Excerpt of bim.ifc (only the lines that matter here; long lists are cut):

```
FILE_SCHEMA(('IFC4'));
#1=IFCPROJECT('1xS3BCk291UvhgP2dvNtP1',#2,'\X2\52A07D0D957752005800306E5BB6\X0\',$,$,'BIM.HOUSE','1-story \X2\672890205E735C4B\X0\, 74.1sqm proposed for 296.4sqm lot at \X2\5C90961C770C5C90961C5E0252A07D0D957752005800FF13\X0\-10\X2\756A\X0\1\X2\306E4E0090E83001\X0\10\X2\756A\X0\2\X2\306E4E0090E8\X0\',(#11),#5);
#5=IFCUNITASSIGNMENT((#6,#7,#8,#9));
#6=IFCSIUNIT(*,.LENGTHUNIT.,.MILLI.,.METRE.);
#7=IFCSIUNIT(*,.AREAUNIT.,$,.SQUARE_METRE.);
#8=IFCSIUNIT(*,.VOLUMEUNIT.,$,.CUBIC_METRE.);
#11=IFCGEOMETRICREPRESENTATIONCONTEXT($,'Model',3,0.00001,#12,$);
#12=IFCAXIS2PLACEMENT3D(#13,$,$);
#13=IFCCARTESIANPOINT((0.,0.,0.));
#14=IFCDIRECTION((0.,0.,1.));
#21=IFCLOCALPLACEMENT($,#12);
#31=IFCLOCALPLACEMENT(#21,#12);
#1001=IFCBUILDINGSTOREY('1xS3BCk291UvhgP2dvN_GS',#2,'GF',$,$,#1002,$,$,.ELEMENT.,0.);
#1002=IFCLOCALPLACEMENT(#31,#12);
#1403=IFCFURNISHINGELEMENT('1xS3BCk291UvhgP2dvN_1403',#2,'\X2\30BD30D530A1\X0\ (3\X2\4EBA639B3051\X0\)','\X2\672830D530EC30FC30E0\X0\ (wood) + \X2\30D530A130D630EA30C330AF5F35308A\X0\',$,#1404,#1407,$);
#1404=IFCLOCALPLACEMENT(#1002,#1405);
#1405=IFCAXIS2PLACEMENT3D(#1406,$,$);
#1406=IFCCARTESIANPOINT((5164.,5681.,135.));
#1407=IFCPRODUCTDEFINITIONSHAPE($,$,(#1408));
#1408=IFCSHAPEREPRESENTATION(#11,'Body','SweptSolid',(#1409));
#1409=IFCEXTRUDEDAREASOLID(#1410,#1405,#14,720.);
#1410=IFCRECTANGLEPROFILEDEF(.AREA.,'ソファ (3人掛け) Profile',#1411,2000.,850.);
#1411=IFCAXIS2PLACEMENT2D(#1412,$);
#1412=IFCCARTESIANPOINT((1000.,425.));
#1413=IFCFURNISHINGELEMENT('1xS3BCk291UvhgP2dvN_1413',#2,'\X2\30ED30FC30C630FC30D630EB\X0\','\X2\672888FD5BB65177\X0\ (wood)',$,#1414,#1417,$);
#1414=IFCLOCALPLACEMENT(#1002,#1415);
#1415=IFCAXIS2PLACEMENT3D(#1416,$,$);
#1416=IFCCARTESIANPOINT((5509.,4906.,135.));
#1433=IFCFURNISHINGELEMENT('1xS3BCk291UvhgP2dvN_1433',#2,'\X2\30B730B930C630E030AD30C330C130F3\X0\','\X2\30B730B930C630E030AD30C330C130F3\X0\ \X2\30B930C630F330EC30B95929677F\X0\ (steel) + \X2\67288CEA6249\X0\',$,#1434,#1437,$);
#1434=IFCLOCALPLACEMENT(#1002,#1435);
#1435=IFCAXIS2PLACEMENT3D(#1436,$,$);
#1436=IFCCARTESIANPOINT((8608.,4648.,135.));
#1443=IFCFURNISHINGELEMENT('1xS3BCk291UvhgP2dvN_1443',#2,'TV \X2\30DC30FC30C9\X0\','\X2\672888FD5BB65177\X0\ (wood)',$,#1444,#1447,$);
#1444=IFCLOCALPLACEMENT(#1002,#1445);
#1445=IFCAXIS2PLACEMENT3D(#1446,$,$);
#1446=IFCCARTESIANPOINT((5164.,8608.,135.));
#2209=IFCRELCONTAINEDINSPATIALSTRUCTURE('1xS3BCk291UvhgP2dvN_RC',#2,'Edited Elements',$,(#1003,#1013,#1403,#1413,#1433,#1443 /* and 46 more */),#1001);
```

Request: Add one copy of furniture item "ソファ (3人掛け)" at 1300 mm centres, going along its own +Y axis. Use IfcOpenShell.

```python
import ifcopenshell
import ifcopenshell.api.geometry
import ifcopenshell.api.root
import ifcopenshell.util.element
import ifcopenshell.util.placement
import ifcopenshell.util.unit

model = ifcopenshell.open("bim.ifc")
unit_scale = ifcopenshell.util.unit.calculate_unit_scale(model)


def reuse_history(source, copy):
    """copy_class also copies each property set's owner history, people and application; keep the originals."""
    for rel in copy.IsDefinedBy:
        if rel.is_a("IfcRelDefinesByProperties") and (history := rel.RelatingPropertyDefinition.OwnerHistory):
            rel.RelatingPropertyDefinition.OwnerHistory = source.OwnerHistory
            ifcopenshell.util.element.remove_deep2(model, history)


source = model.by_guid("1xS3BCk291UvhgP2dvN_1403")
base = ifcopenshell.util.placement.get_local_placement(source.ObjectPlacement)
step = base[:3, 1] * 1.3 / unit_scale

for i in range(1, 2):
    copy = ifcopenshell.api.root.copy_class(model, product=source)
    copy.Representation = ifcopenshell.util.element.copy_deep(
        model, source.Representation, exclude=["IfcGeometricRepresentationContext", "IfcRepresentationMap"]
    )
    reuse_history(source, copy)
    matrix = base.copy()
    matrix[:3, 3] += i * step
    print("added at", matrix[:3, 3].round(3) + 0.0)
    ifcopenshell.api.geometry.edit_object_placement(model, product=copy, matrix=matrix, is_si=False)

model.write("bim-out.ifc")
```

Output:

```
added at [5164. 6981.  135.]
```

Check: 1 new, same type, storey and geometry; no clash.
